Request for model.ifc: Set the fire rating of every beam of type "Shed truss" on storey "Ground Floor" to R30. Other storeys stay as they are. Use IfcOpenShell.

First a look at what the model holds.

```python
import ifcopenshell
import ifcopenshell.util.element

model = ifcopenshell.open("model.ifc")
print(model.schema)
storey = next(s for s in model.by_type("IfcBuildingStorey") if s.Name == "Ground Floor")
beams = [e for e in ifcopenshell.util.element.get_decomposition(storey) if e.is_a("IfcBeam")]
seen = {}
for e in beams:
    element_type = ifcopenshell.util.element.get_type(e)
    key = (element_type.Name if element_type != e and element_type else None, ifcopenshell.util.element.get_pset(e, "Pset_BeamCommon", "FireRating"))
    seen[key] = seen.get(key, 0) + 1
for (name, value), count in sorted(seen.items(), key=str):
    print(count, "x", name, "|", value)
```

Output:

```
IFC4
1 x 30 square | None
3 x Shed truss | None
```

```python
import ifcopenshell
import ifcopenshell.api.pset
import ifcopenshell.util.element

model = ifcopenshell.open("model.ifc")

storey = next(s for s in model.by_type("IfcBuildingStorey") if s.Name == "Ground Floor")
beams = [e for e in ifcopenshell.util.element.get_decomposition(storey) if e.is_a("IfcBeam")]

count = 0
for e in beams:
    element_type = ifcopenshell.util.element.get_type(e)
    if element_type in (None, e) or element_type.Name != "Shed truss":
        continue
    # add_pset returns the element's existing set when there is one.
    pset = ifcopenshell.api.pset.add_pset(model, product=e, name="Pset_BeamCommon")
    ifcopenshell.api.pset.edit_pset(model, pset=pset, properties={"FireRating": "R30"})
    count += 1

print(count, "beams updated")

model.write("model_v2.ifc")
```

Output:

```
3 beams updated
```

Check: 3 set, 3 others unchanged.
